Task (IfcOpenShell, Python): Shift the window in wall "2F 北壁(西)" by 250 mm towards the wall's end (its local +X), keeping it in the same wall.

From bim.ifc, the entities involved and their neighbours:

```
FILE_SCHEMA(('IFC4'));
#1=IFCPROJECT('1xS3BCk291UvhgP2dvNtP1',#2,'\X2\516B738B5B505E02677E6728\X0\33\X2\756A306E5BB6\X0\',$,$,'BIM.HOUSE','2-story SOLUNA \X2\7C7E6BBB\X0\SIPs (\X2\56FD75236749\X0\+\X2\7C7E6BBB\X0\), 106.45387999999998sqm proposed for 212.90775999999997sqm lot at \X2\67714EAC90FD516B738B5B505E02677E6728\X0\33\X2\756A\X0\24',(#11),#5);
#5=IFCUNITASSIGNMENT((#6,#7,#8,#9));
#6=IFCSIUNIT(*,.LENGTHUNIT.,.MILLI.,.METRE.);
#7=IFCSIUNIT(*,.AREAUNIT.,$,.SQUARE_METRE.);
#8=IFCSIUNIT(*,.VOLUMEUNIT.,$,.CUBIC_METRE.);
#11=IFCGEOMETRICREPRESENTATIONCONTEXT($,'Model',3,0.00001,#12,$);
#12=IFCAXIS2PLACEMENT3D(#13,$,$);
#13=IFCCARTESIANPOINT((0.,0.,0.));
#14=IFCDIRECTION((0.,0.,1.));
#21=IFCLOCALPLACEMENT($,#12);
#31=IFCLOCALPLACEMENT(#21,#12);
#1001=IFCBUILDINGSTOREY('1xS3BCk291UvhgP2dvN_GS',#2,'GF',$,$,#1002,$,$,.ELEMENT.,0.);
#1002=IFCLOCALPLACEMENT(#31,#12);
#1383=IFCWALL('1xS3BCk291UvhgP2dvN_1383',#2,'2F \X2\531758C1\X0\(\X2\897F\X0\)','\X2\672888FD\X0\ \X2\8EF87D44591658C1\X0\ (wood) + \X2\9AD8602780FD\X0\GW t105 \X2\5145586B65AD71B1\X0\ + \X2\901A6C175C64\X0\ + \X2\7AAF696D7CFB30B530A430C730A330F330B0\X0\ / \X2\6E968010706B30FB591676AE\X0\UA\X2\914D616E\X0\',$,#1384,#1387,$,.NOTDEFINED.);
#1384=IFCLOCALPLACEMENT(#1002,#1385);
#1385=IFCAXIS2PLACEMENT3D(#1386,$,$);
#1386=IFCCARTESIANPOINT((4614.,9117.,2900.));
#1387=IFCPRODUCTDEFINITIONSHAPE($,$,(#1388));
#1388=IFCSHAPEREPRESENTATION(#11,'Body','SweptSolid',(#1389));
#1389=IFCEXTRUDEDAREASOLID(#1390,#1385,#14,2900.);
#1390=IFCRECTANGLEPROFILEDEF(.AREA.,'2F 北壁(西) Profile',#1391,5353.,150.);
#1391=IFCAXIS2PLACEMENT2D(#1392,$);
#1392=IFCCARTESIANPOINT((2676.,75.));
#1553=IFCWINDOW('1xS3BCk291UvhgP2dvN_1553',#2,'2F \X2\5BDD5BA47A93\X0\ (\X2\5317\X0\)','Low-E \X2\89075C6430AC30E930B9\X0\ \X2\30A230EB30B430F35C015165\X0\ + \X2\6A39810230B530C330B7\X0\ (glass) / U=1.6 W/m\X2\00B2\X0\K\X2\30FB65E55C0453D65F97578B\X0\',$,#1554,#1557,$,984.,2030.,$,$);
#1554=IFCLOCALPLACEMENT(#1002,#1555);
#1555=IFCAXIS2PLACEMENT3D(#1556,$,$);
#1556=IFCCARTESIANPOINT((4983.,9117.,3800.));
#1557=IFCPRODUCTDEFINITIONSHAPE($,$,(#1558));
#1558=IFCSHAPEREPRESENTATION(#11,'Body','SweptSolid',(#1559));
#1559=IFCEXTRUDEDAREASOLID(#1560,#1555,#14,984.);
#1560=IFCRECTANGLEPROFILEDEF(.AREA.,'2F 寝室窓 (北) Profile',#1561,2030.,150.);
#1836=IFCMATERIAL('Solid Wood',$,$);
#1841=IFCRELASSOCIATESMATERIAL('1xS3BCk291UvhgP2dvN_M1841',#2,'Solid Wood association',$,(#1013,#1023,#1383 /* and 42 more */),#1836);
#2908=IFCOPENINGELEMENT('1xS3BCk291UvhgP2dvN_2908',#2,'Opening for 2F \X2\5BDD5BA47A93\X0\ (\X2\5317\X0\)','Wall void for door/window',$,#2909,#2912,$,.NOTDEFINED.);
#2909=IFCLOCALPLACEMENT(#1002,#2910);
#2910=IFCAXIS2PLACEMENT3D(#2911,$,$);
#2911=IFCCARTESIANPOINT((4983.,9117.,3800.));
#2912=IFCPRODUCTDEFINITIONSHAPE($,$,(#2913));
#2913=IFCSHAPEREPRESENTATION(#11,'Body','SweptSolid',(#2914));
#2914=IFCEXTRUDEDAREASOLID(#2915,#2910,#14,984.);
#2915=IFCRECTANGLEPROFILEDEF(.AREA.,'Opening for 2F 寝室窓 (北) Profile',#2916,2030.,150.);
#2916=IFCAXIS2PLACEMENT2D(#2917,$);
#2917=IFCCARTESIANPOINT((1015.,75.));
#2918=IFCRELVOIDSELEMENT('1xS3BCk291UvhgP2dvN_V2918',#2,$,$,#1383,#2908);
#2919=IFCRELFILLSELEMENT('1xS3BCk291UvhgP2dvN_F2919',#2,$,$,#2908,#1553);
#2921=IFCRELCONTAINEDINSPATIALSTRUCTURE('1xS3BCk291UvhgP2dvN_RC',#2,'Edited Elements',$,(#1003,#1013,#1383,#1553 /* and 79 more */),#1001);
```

```python
import ifcopenshell
import ifcopenshell.api.geometry
import ifcopenshell.util.placement

model = ifcopenshell.open("bim.ifc")

window = model.by_guid("1xS3BCk291UvhgP2dvN_1553")
opening = window.FillsVoids[0].RelatingOpeningElement
wall = opening.VoidsElements[0].RelatingBuildingElement

wall_matrix = ifcopenshell.util.placement.get_local_placement(wall.ObjectPlacement)
shift = wall_matrix[:3, 0] * 250.0
before = ifcopenshell.util.placement.get_local_placement(window.ObjectPlacement)[:3, 3].copy()

# The window is not placed relative to its opening, so move both.
for product in (opening, window):
    matrix = ifcopenshell.util.placement.get_local_placement(product.ObjectPlacement)
    matrix[:3, 3] += shift
    ifcopenshell.api.geometry.edit_object_placement(model, product=product, matrix=matrix, is_si=False)

after = ifcopenshell.util.placement.get_local_placement(window.ObjectPlacement)[:3, 3]
print("window moved by", (after - before).round(3) + 0.0)

model.write("bim_rev.ifc")
```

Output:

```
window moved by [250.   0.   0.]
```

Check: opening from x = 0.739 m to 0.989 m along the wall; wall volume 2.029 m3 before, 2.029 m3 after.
